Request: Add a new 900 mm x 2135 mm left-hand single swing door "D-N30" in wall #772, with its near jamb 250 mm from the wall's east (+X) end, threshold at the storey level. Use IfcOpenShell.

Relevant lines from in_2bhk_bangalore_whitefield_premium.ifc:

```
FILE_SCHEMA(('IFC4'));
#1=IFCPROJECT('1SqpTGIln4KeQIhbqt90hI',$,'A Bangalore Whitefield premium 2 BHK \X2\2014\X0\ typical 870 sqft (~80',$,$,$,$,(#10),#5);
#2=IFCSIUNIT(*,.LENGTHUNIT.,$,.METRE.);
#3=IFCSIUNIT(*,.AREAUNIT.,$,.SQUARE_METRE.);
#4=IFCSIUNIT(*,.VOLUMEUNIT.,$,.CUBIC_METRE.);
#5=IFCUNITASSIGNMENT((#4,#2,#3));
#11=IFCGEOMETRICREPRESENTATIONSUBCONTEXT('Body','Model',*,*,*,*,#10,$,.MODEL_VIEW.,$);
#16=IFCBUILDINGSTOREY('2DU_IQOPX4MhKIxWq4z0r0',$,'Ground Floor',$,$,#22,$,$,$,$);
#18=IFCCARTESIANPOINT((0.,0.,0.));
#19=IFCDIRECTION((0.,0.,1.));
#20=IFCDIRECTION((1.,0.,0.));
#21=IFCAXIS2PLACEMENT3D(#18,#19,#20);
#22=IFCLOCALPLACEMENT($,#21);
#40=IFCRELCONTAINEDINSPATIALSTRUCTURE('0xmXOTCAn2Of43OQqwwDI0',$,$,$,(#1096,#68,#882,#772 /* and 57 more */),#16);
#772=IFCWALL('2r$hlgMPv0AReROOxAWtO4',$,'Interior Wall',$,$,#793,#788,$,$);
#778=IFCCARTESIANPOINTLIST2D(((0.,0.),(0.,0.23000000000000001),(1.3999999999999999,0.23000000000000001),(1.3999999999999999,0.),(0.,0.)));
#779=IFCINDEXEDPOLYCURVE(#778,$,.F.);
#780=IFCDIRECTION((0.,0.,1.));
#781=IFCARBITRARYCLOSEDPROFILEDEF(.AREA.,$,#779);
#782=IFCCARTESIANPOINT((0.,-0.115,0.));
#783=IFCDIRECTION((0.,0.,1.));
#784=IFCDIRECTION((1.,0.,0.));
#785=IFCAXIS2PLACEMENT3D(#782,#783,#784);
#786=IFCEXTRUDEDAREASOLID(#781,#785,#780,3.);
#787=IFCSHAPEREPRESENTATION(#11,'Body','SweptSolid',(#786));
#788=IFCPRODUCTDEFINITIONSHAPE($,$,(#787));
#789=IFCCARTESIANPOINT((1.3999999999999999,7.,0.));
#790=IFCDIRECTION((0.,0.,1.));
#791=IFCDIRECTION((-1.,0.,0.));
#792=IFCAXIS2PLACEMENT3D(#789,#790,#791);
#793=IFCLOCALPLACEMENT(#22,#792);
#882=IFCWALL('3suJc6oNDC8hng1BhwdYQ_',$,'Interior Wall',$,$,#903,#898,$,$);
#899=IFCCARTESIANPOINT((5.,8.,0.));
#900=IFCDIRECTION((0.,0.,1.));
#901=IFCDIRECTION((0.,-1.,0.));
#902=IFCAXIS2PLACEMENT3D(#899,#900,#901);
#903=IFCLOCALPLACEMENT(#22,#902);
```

```python
import numpy as np
import ifcopenshell
import ifcopenshell.api.feature
import ifcopenshell.api.geometry
import ifcopenshell.api.root
import ifcopenshell.api.spatial
import ifcopenshell.geom
import ifcopenshell.util.element
import ifcopenshell.util.placement
import ifcopenshell.util.representation
import ifcopenshell.util.shape
import ifcopenshell.util.unit

model = ifcopenshell.open("in_2bhk_bangalore_whitefield_premium.ifc")
unit_scale = ifcopenshell.util.unit.calculate_unit_scale(model)
settings = ifcopenshell.geom.settings()


def volume(element):
    """Net volume in cubic metres, openings subtracted."""
    shape = ifcopenshell.geom.create_shape(settings, element)
    return ifcopenshell.util.shape.get_volume(shape.geometry)


wall = model.by_guid("2r$hlgMPv0AReROOxAWtO4")
storey = ifcopenshell.util.element.get_container(wall, ifc_class="IfcBuildingStorey")
context = ifcopenshell.util.representation.get_context(model, "Model", "Body", "MODEL_VIEW")
before = volume(wall)

width, height, from_end, sill = 0.9, 2.135, 0.25, 0.0  # metres

# The wall runs along its own X axis, and the end named is its -X end.
wall_shape = ifcopenshell.geom.create_shape(settings, wall)
x, y, z = ifcopenshell.util.shape.get_vertices(wall_shape.geometry).T
start = x.min() + from_end
face, thickness = float(y.min()), float(y.max() - y.min())
wall_matrix = ifcopenshell.util.placement.get_local_placement(wall.ObjectPlacement)
level = ifcopenshell.util.placement.get_local_placement(storey.ObjectPlacement)[2, 3]


def in_wall(x, y):
    """Placement at x, y metres in the wall's axes, at sill height."""
    matrix = wall_matrix.copy()
    matrix[:, 3] = wall_matrix @ np.array([x / unit_scale, y / unit_scale, 0.0, 1.0])
    matrix[2, 3] = level + sill / unit_scale
    return matrix


# Opening: a box that overshoots both wall faces by 50 mm.
opening = ifcopenshell.api.root.create_entity(model, ifc_class="IfcOpeningElement", predefined_type="OPENING")
box = ifcopenshell.api.geometry.add_wall_representation(
    model, context=context, length=width, height=height, thickness=thickness + 0.1
)
ifcopenshell.api.geometry.assign_representation(model, product=opening, representation=box)
ifcopenshell.api.geometry.edit_object_placement(model, product=opening, matrix=in_wall(start, face - 0.05), is_si=False)
ifcopenshell.api.feature.add_feature(model, feature=opening, element=wall)

door = ifcopenshell.api.root.create_entity(model, ifc_class="IfcDoor", name="D-N30", predefined_type="DOOR")
door.OverallWidth, door.OverallHeight = width / unit_scale, height / unit_scale
door.OperationType = "SINGLE_SWING_LEFT"
body = ifcopenshell.api.geometry.add_door_representation(
    model,
    context=context,
    overall_width=door.OverallWidth,
    overall_height=door.OverallHeight,
    operation_type="SINGLE_SWING_LEFT",
    lining_properties={"LiningDepth": thickness / unit_scale, "ThresholdDepth": thickness / unit_scale},
)
ifcopenshell.api.geometry.assign_representation(model, product=door, representation=body)
ifcopenshell.api.spatial.assign_container(model, products=[door], relating_structure=storey)
ifcopenshell.api.feature.add_filling(model, opening=opening, element=door)

# The lining spans the wall, so the door starts at the wall face.
ifcopenshell.api.geometry.edit_object_placement(model, product=door, matrix=in_wall(start, face), is_si=False)

after = volume(wall)

print(f"wall volume {before:.3f} -> {after:.3f} m3")

model.write("in_2bhk_bangalore_whitefield_premium_rev.ifc")
```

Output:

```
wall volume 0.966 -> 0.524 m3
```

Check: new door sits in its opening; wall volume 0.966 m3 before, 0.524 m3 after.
